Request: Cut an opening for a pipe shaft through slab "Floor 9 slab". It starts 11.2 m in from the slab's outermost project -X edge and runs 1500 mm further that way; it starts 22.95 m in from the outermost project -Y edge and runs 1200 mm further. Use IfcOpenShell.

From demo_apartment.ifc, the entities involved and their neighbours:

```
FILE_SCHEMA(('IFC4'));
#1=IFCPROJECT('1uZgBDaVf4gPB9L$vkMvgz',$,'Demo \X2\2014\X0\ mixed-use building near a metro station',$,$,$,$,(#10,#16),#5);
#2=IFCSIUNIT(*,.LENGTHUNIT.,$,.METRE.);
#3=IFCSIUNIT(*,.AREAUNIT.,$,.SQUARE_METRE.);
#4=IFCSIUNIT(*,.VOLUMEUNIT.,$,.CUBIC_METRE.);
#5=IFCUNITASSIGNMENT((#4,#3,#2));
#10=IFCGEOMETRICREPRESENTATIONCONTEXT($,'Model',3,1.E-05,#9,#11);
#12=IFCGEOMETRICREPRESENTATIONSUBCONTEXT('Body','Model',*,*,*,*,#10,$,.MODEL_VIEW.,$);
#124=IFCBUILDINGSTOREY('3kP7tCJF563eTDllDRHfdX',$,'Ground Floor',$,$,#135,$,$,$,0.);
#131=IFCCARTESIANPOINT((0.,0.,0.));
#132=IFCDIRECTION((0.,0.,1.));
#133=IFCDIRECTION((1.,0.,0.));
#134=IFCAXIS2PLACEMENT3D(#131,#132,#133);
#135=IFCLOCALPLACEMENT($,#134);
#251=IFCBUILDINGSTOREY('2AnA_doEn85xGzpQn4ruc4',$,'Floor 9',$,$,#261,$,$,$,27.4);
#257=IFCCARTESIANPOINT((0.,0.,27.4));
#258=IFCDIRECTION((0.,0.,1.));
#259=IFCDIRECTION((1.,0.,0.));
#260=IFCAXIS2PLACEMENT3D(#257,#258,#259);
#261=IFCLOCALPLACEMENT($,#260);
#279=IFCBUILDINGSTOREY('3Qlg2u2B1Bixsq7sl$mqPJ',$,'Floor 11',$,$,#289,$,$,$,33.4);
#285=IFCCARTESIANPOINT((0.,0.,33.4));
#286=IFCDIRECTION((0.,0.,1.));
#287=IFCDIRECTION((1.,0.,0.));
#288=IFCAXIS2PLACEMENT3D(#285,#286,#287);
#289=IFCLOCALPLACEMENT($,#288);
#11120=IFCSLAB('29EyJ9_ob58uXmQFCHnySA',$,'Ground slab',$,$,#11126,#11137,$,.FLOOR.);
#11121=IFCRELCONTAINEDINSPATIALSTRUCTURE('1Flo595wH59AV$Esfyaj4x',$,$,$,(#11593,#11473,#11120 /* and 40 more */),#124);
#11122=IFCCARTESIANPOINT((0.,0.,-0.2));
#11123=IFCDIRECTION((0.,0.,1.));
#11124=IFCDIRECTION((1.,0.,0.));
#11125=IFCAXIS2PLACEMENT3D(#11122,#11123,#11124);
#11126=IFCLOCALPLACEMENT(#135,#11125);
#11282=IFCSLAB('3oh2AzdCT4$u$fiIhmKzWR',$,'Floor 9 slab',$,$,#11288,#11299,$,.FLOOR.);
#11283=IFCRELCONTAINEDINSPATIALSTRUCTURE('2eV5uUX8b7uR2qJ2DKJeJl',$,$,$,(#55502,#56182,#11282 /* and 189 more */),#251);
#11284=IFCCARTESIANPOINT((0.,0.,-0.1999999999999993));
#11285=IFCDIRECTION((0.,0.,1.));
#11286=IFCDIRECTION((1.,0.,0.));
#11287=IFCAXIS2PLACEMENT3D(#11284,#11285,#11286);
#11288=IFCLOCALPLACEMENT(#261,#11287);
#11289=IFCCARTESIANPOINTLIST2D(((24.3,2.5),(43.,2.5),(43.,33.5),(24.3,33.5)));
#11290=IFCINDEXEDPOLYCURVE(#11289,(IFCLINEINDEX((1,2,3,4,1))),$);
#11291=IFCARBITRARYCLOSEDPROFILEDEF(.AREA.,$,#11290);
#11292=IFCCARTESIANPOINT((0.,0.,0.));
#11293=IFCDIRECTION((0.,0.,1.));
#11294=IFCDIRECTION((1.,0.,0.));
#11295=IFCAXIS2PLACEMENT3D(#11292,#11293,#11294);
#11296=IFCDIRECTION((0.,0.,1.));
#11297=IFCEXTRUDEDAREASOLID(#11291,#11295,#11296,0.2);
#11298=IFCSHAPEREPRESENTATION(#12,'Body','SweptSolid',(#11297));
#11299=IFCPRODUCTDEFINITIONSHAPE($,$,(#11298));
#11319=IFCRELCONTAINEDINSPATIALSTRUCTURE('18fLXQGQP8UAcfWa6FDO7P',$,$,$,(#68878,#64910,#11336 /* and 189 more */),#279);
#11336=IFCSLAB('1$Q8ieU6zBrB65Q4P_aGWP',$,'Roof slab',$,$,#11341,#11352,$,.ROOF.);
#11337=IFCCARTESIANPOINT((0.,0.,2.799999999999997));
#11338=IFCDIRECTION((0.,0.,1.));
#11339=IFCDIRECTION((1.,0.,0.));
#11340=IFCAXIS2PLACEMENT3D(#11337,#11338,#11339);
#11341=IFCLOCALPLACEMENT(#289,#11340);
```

```python
import numpy as np
import ifcopenshell
import ifcopenshell.api.feature
import ifcopenshell.api.geometry
import ifcopenshell.api.root
import ifcopenshell.geom
import ifcopenshell.util.placement
import ifcopenshell.util.representation
import ifcopenshell.util.shape
import ifcopenshell.util.unit

model = ifcopenshell.open("demo_apartment.ifc")
unit_scale = ifcopenshell.util.unit.calculate_unit_scale(model)
settings = ifcopenshell.geom.settings()


def volume(element):
    """Net volume in cubic metres, openings subtracted."""
    shape = ifcopenshell.geom.create_shape(settings, element)
    return ifcopenshell.util.shape.get_volume(shape.geometry)


slab = model.by_guid("3oh2AzdCT4$u$fiIhmKzWR")
before = volume(slab)

# Extent in the slab's own axes, in metres. The edges named are its -X and -Y sides.
slab_shape = ifcopenshell.geom.create_shape(settings, slab)
vertices = ifcopenshell.util.shape.get_vertices(slab_shape.geometry)
x_min, y_min, bottom = vertices.min(axis=0)
top = vertices[:, 2].max()

opening = ifcopenshell.api.root.create_entity(model, ifc_class="IfcOpeningElement", name="Pipe shaft opening", predefined_type="OPENING")
context = ifcopenshell.util.representation.get_context(model, "Model", "Body", "MODEL_VIEW")
width, depth = 1.5, 1.2
outline = [(0.0, 0.0), (width, 0.0), (width, depth), (0.0, depth), (0.0, 0.0)]
# Overshoot both faces by 50 mm so the cut is clean.
shape = ifcopenshell.api.geometry.add_slab_representation(
    model, context=context, depth=top - bottom + 0.1, polyline=outline
)
ifcopenshell.api.geometry.assign_representation(model, product=opening, representation=shape)

matrix = ifcopenshell.util.placement.get_local_placement(slab.ObjectPlacement)
matrix[:, 3] = matrix @ np.append(np.array([x_min + 11.2, y_min + 22.95, bottom - 0.05]) / unit_scale, 1.0)
ifcopenshell.api.geometry.edit_object_placement(model, product=opening, matrix=matrix, is_si=False)
ifcopenshell.api.feature.add_feature(model, feature=opening, element=slab)

after = volume(slab)

print(f"slab volume {before:.3f} -> {after:.3f} m3")

model.write("demo_apartment_edited.ifc")
```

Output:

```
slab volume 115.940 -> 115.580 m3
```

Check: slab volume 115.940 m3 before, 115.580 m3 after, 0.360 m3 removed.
